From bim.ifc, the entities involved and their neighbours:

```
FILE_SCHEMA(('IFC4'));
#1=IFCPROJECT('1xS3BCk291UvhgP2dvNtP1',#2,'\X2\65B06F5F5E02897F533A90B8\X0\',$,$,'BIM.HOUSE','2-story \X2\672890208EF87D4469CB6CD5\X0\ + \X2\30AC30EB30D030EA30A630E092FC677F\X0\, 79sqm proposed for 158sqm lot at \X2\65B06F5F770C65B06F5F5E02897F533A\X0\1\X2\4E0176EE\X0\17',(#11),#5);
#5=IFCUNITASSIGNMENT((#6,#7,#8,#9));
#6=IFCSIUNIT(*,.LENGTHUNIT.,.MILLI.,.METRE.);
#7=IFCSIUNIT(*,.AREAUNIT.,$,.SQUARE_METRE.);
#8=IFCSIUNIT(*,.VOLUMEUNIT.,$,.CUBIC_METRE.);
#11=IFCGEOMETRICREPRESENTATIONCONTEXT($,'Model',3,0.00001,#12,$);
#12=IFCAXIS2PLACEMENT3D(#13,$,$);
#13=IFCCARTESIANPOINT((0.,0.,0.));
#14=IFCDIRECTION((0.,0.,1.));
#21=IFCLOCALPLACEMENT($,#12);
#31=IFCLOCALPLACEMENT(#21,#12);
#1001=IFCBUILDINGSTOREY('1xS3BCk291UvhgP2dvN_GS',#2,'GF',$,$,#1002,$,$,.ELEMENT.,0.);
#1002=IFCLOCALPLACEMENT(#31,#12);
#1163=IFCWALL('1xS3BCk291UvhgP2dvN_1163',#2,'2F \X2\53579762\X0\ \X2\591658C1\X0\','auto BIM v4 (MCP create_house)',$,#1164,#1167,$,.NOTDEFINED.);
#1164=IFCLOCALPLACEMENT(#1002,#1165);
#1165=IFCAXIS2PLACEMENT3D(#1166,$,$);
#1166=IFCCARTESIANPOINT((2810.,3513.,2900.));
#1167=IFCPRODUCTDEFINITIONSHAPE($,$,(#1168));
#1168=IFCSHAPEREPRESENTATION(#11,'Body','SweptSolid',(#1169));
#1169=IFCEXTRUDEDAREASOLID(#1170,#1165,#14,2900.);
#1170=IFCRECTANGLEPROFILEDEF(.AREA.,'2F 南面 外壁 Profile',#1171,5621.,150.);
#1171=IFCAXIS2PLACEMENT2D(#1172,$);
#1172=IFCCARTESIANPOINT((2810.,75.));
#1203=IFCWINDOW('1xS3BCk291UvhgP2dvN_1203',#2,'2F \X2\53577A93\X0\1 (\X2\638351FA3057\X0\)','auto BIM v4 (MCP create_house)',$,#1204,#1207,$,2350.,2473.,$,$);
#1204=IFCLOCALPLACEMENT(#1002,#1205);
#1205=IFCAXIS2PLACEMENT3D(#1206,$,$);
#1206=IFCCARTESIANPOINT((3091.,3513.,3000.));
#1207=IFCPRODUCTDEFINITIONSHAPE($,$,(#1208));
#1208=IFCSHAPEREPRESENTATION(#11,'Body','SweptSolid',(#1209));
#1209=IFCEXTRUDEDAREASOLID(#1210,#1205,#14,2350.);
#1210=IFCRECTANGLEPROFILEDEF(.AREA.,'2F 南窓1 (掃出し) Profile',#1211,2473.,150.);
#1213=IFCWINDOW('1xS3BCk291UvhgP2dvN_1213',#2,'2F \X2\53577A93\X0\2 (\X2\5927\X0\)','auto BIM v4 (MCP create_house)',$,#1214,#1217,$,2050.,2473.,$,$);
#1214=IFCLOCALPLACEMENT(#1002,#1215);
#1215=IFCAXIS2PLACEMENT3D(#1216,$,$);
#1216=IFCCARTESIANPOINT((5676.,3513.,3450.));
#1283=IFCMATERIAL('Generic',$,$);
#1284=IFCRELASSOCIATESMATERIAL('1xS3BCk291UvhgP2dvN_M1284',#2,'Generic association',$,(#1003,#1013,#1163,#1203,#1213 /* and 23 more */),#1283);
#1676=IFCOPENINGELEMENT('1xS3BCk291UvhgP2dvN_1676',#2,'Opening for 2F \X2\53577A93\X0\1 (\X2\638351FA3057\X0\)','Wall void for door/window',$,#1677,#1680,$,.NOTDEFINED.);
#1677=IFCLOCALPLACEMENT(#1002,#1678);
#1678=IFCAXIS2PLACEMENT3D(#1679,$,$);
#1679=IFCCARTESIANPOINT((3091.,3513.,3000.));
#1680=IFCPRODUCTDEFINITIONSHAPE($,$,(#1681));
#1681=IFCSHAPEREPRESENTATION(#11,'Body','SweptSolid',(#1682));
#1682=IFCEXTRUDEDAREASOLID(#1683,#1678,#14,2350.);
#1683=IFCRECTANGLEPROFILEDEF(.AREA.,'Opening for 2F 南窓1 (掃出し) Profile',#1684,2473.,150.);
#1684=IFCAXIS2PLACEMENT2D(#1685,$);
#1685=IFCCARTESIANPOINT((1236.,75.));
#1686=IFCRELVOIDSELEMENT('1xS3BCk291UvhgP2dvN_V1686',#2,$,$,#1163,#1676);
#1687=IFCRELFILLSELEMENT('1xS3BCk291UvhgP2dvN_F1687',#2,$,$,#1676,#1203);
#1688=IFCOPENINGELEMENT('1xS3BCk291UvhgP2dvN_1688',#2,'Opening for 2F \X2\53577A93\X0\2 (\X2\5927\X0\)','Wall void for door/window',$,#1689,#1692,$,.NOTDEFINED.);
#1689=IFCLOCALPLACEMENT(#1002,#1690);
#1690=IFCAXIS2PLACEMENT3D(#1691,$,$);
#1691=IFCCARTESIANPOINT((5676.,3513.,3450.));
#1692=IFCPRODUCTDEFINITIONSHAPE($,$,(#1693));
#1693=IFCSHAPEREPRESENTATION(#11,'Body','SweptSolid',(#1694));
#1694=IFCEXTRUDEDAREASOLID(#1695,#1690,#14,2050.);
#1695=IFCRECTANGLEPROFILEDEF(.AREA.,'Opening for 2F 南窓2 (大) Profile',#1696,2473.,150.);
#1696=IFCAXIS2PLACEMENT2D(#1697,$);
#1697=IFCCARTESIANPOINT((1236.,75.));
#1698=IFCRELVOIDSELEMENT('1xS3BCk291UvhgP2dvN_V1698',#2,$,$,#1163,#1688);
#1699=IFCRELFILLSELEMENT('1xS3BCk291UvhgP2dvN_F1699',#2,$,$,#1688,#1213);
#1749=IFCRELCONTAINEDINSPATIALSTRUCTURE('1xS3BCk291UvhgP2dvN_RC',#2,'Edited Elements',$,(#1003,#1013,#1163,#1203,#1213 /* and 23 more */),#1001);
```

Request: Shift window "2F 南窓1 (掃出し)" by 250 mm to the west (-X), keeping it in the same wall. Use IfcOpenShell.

```python
import ifcopenshell
import ifcopenshell.api.geometry
import ifcopenshell.util.placement

model = ifcopenshell.open("bim.ifc")

window = model.by_guid("1xS3BCk291UvhgP2dvN_1203")
opening = window.FillsVoids[0].RelatingOpeningElement
wall = opening.VoidsElements[0].RelatingBuildingElement

wall_matrix = ifcopenshell.util.placement.get_local_placement(wall.ObjectPlacement)
shift = wall_matrix[:3, 0] * -250.0
before = ifcopenshell.util.placement.get_local_placement(window.ObjectPlacement)[:3, 3].copy()

# The window is not placed relative to its opening, so move both.
for product in (opening, window):
    matrix = ifcopenshell.util.placement.get_local_placement(product.ObjectPlacement)
    matrix[:3, 3] += shift
    ifcopenshell.api.geometry.edit_object_placement(model, product=product, matrix=matrix, is_si=False)

after = ifcopenshell.util.placement.get_local_placement(window.ObjectPlacement)[:3, 3]
print("window moved by", (after - before).round(3) + 0.0)

model.write("bim_rev.ifc")
```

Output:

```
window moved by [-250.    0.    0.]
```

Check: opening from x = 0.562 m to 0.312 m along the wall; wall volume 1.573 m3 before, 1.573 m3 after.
